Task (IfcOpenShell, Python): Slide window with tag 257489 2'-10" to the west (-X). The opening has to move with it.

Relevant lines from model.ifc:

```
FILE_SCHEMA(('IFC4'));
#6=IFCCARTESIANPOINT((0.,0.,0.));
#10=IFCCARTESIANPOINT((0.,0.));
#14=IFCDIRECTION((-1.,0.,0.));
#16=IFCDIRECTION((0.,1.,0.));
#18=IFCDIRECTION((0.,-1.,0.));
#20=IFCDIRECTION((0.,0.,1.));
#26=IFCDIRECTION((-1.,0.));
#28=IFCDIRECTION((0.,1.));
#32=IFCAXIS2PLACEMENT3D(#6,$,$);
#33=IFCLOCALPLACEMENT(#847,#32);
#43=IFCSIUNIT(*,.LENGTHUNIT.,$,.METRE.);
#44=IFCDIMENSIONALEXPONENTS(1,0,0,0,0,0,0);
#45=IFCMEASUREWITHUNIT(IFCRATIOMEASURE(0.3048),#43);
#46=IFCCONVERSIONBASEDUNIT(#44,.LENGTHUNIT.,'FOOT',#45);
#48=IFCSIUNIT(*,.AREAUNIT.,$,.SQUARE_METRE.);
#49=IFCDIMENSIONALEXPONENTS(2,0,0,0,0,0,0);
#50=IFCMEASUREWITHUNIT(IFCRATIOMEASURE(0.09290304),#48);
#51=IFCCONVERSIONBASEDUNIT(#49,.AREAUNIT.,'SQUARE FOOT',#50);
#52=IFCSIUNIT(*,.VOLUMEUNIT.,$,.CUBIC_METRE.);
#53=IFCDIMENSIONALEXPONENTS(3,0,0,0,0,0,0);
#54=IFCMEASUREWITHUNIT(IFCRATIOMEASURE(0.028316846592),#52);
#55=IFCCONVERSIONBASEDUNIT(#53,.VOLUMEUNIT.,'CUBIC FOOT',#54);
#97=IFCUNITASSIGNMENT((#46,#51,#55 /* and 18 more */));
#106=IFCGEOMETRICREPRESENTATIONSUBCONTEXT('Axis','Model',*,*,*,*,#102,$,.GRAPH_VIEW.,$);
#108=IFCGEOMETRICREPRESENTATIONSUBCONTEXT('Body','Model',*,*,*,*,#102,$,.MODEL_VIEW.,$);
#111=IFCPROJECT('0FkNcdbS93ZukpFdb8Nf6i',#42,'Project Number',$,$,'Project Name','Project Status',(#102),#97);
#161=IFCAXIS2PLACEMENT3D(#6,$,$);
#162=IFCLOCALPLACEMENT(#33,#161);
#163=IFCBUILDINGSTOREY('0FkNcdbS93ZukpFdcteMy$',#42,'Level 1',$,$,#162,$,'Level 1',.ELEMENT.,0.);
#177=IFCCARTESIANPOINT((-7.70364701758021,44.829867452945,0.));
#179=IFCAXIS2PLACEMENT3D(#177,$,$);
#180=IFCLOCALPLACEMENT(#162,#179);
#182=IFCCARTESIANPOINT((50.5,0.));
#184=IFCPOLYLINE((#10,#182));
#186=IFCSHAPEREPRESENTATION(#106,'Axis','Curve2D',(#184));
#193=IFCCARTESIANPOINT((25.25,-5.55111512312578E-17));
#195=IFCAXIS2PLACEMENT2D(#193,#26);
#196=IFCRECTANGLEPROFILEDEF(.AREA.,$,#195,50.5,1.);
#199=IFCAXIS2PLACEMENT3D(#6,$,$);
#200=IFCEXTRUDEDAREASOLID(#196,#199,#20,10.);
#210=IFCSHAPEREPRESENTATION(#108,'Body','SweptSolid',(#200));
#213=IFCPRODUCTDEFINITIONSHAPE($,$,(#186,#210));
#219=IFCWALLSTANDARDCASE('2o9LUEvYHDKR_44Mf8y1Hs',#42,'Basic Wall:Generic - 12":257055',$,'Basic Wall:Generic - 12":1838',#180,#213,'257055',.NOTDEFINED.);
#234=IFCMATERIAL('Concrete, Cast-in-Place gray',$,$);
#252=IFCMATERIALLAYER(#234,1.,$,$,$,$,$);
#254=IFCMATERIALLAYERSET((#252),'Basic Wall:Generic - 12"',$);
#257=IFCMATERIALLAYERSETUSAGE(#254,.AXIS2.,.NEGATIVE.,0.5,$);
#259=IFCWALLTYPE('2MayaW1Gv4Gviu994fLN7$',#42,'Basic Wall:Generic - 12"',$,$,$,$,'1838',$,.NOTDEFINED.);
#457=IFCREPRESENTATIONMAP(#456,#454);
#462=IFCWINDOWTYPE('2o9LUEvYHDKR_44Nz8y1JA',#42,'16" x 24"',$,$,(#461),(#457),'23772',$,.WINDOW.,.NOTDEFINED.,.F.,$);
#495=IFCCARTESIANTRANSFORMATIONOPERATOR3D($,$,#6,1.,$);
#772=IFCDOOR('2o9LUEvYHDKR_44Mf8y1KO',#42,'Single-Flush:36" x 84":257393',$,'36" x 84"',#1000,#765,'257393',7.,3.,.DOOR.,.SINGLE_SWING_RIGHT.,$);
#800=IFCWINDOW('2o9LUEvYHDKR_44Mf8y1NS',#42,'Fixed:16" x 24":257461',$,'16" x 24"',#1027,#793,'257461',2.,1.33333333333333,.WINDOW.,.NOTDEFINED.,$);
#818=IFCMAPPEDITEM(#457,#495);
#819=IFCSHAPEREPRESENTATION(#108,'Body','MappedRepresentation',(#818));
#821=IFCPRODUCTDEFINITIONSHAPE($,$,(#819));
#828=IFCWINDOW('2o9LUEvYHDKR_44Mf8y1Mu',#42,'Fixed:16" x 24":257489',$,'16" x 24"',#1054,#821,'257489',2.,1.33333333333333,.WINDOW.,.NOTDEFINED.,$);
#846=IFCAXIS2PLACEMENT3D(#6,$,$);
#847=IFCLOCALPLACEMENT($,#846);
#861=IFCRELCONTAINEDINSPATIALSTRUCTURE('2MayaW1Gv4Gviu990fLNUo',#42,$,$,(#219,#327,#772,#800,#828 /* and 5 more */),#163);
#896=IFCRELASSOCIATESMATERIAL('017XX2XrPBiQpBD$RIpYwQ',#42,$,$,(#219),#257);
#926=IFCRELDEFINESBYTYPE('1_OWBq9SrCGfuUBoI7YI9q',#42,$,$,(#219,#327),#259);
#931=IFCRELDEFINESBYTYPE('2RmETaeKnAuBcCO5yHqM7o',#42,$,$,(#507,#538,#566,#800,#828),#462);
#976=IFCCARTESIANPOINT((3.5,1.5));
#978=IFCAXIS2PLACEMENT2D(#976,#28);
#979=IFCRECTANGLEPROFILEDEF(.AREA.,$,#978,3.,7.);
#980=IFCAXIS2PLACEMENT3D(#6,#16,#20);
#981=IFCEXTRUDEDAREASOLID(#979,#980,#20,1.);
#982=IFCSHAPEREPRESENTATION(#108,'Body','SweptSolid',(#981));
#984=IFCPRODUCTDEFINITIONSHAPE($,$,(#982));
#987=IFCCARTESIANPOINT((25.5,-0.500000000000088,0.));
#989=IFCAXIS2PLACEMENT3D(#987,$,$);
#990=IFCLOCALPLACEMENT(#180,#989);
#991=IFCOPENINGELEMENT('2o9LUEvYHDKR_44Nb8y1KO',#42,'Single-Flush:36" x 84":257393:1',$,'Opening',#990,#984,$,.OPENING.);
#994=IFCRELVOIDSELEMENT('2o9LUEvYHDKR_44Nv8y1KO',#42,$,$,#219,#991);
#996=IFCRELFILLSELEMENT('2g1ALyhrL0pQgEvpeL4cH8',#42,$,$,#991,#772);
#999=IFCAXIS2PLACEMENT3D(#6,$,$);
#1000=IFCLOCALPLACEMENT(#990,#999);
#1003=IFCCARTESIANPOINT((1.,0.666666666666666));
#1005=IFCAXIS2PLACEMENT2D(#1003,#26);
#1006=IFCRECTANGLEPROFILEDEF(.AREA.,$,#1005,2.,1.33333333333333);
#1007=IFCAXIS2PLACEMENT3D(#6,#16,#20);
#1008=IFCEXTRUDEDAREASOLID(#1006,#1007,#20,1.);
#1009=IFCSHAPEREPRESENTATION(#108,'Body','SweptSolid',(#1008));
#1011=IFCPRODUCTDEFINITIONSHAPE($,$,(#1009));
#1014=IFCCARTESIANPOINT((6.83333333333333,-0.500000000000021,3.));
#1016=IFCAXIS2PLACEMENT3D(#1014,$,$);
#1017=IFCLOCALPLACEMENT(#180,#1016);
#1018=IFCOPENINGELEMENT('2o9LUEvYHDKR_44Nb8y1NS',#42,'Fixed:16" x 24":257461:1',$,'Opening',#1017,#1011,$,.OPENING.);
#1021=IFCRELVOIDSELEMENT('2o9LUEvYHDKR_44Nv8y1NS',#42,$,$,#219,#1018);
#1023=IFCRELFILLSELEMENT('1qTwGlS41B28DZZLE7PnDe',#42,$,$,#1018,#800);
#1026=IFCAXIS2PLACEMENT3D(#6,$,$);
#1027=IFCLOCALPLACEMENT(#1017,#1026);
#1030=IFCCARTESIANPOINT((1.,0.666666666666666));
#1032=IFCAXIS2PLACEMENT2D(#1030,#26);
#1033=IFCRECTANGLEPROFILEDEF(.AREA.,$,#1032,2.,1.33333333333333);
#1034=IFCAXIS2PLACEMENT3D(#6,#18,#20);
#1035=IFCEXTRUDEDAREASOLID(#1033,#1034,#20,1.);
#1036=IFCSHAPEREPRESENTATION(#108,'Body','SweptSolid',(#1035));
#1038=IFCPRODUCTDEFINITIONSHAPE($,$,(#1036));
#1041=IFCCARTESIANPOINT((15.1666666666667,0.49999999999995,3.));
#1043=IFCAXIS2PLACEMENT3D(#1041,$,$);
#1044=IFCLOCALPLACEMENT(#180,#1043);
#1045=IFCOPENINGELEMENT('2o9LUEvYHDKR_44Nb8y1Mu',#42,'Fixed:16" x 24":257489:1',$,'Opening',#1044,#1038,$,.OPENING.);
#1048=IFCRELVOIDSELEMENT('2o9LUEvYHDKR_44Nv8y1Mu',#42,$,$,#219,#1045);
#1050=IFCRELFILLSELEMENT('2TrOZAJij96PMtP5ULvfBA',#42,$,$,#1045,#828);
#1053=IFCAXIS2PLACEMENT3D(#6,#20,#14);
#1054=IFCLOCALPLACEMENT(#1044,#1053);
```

```python
import ifcopenshell
import ifcopenshell.api.geometry
import ifcopenshell.util.placement
import ifcopenshell.util.unit

model = ifcopenshell.open("model.ifc")
unit_scale = ifcopenshell.util.unit.calculate_unit_scale(model)

window = model.by_guid("2o9LUEvYHDKR_44Mf8y1Mu")
opening = window.FillsVoids[0].RelatingOpeningElement
wall = opening.VoidsElements[0].RelatingBuildingElement

wall_matrix = ifcopenshell.util.placement.get_local_placement(wall.ObjectPlacement)
shift = wall_matrix[:3, 0] * -34 * 0.0254 / unit_scale
before = ifcopenshell.util.placement.get_local_placement(window.ObjectPlacement)[:3, 3].copy()

# The window is placed relative to its opening, so it follows when the opening moves.
matrix = ifcopenshell.util.placement.get_local_placement(opening.ObjectPlacement)
matrix[:3, 3] += shift
ifcopenshell.api.geometry.edit_object_placement(
    model, product=opening, matrix=matrix, is_si=False, should_transform_children=True
)

after = ifcopenshell.util.placement.get_local_placement(window.ObjectPlacement)[:3, 3]
print("window moved by", (after - before).round(3) + 0.0)

model.write("model-out.ifc")
```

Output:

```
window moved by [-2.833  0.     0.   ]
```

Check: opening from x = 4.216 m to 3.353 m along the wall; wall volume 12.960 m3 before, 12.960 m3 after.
